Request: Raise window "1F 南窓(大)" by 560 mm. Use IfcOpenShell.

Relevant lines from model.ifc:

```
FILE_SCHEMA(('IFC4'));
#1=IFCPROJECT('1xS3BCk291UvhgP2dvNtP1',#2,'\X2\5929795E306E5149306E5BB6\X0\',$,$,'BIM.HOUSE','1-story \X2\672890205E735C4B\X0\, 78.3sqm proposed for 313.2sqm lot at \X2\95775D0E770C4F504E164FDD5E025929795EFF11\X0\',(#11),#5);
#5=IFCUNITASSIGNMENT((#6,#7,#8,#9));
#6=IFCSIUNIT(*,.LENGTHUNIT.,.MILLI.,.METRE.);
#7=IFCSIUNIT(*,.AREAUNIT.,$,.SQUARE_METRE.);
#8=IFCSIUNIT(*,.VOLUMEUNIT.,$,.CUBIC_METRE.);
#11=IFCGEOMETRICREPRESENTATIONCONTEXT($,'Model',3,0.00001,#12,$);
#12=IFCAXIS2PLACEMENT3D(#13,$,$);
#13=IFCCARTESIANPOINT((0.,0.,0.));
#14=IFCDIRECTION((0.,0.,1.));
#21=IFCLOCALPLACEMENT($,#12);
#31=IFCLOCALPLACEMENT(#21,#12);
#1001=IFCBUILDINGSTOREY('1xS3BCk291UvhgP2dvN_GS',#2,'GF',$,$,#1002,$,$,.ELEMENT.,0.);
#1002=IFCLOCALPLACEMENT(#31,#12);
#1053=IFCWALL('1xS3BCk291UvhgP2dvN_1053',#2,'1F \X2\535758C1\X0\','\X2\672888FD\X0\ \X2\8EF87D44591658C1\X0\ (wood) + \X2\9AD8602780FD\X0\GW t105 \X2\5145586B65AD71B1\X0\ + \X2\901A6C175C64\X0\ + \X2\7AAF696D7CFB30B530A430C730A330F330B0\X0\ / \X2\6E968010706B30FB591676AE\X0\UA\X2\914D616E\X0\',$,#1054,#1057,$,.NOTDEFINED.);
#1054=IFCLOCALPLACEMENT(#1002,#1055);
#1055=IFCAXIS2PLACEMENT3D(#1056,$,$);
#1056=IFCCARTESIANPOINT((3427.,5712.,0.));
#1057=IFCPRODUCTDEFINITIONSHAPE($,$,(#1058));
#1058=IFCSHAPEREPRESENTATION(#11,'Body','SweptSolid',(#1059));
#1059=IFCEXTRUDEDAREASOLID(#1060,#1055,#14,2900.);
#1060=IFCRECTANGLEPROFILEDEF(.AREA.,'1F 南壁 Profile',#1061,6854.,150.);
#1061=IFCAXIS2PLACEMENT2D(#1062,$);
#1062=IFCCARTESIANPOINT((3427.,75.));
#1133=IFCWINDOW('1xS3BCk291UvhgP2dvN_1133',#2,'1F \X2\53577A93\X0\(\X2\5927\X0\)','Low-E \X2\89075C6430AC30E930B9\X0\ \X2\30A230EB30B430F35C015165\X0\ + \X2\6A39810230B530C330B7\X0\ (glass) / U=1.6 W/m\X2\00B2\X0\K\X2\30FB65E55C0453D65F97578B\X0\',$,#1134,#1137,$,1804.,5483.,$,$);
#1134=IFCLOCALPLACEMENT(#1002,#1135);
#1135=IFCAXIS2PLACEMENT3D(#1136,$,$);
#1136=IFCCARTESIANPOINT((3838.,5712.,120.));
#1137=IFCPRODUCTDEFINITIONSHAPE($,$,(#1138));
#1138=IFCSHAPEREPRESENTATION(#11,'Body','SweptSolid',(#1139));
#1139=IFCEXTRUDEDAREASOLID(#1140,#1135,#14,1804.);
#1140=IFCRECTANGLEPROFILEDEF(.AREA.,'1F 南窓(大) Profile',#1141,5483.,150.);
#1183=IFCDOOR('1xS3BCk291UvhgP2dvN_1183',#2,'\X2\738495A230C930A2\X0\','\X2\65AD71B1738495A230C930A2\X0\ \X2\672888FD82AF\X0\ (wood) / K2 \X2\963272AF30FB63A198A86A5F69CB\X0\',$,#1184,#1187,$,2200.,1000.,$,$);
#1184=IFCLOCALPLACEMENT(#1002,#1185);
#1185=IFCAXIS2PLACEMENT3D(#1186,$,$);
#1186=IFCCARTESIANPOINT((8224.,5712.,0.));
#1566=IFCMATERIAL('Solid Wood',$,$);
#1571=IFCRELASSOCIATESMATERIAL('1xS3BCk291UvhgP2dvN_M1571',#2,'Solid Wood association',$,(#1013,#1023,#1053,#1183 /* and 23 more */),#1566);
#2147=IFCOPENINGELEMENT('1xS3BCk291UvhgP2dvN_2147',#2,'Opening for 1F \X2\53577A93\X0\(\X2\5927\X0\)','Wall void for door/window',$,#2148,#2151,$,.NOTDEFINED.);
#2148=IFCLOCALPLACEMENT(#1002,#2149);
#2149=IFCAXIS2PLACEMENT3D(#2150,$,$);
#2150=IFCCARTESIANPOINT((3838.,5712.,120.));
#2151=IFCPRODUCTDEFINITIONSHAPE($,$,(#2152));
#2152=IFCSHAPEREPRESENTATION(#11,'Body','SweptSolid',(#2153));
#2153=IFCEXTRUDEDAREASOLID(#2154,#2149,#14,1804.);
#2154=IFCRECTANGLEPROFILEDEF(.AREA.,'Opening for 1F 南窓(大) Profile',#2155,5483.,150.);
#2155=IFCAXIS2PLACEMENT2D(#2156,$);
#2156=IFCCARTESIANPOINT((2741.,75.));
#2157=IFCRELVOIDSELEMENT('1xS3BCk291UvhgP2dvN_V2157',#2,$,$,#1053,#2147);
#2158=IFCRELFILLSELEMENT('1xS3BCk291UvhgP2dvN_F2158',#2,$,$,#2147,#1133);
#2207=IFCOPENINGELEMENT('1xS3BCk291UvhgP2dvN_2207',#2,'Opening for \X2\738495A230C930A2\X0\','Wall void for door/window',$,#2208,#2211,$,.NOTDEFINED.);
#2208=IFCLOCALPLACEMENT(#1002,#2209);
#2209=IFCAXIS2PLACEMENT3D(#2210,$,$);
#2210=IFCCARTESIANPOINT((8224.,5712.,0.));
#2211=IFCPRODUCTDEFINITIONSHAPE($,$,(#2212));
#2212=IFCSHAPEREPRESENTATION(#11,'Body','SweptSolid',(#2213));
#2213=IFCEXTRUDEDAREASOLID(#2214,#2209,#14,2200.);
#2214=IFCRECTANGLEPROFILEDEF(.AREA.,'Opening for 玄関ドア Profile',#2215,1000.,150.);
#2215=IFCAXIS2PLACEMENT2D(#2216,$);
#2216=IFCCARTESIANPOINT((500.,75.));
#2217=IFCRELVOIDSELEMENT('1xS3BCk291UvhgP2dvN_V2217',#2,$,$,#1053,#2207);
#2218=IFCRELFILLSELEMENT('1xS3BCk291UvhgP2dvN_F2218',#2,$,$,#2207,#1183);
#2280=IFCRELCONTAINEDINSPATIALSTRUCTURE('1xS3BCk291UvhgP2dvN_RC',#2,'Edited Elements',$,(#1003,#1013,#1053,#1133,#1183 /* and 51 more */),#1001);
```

```python
import numpy as np
import ifcopenshell
import ifcopenshell.api.geometry
import ifcopenshell.util.placement
import ifcopenshell.util.unit

model = ifcopenshell.open("model.ifc")
unit_scale = ifcopenshell.util.unit.calculate_unit_scale(model)

window = model.by_guid("1xS3BCk291UvhgP2dvN_1133")
opening = window.FillsVoids[0].RelatingOpeningElement
dz = 0.56 / unit_scale

shift = np.array([0.0, 0.0, dz])
# The window is not placed relative to its opening, so move both.
for product in (opening, window):
    matrix = ifcopenshell.util.placement.get_local_placement(product.ObjectPlacement)
    matrix[:3, 3] += shift
    ifcopenshell.api.geometry.edit_object_placement(model, product=product, matrix=matrix, is_si=False)

print(f"moved by {dz * unit_scale:+.3f} m")

model.write("model_edited.ifc")
```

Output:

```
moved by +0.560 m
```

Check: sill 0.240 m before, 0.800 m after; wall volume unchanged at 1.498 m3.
